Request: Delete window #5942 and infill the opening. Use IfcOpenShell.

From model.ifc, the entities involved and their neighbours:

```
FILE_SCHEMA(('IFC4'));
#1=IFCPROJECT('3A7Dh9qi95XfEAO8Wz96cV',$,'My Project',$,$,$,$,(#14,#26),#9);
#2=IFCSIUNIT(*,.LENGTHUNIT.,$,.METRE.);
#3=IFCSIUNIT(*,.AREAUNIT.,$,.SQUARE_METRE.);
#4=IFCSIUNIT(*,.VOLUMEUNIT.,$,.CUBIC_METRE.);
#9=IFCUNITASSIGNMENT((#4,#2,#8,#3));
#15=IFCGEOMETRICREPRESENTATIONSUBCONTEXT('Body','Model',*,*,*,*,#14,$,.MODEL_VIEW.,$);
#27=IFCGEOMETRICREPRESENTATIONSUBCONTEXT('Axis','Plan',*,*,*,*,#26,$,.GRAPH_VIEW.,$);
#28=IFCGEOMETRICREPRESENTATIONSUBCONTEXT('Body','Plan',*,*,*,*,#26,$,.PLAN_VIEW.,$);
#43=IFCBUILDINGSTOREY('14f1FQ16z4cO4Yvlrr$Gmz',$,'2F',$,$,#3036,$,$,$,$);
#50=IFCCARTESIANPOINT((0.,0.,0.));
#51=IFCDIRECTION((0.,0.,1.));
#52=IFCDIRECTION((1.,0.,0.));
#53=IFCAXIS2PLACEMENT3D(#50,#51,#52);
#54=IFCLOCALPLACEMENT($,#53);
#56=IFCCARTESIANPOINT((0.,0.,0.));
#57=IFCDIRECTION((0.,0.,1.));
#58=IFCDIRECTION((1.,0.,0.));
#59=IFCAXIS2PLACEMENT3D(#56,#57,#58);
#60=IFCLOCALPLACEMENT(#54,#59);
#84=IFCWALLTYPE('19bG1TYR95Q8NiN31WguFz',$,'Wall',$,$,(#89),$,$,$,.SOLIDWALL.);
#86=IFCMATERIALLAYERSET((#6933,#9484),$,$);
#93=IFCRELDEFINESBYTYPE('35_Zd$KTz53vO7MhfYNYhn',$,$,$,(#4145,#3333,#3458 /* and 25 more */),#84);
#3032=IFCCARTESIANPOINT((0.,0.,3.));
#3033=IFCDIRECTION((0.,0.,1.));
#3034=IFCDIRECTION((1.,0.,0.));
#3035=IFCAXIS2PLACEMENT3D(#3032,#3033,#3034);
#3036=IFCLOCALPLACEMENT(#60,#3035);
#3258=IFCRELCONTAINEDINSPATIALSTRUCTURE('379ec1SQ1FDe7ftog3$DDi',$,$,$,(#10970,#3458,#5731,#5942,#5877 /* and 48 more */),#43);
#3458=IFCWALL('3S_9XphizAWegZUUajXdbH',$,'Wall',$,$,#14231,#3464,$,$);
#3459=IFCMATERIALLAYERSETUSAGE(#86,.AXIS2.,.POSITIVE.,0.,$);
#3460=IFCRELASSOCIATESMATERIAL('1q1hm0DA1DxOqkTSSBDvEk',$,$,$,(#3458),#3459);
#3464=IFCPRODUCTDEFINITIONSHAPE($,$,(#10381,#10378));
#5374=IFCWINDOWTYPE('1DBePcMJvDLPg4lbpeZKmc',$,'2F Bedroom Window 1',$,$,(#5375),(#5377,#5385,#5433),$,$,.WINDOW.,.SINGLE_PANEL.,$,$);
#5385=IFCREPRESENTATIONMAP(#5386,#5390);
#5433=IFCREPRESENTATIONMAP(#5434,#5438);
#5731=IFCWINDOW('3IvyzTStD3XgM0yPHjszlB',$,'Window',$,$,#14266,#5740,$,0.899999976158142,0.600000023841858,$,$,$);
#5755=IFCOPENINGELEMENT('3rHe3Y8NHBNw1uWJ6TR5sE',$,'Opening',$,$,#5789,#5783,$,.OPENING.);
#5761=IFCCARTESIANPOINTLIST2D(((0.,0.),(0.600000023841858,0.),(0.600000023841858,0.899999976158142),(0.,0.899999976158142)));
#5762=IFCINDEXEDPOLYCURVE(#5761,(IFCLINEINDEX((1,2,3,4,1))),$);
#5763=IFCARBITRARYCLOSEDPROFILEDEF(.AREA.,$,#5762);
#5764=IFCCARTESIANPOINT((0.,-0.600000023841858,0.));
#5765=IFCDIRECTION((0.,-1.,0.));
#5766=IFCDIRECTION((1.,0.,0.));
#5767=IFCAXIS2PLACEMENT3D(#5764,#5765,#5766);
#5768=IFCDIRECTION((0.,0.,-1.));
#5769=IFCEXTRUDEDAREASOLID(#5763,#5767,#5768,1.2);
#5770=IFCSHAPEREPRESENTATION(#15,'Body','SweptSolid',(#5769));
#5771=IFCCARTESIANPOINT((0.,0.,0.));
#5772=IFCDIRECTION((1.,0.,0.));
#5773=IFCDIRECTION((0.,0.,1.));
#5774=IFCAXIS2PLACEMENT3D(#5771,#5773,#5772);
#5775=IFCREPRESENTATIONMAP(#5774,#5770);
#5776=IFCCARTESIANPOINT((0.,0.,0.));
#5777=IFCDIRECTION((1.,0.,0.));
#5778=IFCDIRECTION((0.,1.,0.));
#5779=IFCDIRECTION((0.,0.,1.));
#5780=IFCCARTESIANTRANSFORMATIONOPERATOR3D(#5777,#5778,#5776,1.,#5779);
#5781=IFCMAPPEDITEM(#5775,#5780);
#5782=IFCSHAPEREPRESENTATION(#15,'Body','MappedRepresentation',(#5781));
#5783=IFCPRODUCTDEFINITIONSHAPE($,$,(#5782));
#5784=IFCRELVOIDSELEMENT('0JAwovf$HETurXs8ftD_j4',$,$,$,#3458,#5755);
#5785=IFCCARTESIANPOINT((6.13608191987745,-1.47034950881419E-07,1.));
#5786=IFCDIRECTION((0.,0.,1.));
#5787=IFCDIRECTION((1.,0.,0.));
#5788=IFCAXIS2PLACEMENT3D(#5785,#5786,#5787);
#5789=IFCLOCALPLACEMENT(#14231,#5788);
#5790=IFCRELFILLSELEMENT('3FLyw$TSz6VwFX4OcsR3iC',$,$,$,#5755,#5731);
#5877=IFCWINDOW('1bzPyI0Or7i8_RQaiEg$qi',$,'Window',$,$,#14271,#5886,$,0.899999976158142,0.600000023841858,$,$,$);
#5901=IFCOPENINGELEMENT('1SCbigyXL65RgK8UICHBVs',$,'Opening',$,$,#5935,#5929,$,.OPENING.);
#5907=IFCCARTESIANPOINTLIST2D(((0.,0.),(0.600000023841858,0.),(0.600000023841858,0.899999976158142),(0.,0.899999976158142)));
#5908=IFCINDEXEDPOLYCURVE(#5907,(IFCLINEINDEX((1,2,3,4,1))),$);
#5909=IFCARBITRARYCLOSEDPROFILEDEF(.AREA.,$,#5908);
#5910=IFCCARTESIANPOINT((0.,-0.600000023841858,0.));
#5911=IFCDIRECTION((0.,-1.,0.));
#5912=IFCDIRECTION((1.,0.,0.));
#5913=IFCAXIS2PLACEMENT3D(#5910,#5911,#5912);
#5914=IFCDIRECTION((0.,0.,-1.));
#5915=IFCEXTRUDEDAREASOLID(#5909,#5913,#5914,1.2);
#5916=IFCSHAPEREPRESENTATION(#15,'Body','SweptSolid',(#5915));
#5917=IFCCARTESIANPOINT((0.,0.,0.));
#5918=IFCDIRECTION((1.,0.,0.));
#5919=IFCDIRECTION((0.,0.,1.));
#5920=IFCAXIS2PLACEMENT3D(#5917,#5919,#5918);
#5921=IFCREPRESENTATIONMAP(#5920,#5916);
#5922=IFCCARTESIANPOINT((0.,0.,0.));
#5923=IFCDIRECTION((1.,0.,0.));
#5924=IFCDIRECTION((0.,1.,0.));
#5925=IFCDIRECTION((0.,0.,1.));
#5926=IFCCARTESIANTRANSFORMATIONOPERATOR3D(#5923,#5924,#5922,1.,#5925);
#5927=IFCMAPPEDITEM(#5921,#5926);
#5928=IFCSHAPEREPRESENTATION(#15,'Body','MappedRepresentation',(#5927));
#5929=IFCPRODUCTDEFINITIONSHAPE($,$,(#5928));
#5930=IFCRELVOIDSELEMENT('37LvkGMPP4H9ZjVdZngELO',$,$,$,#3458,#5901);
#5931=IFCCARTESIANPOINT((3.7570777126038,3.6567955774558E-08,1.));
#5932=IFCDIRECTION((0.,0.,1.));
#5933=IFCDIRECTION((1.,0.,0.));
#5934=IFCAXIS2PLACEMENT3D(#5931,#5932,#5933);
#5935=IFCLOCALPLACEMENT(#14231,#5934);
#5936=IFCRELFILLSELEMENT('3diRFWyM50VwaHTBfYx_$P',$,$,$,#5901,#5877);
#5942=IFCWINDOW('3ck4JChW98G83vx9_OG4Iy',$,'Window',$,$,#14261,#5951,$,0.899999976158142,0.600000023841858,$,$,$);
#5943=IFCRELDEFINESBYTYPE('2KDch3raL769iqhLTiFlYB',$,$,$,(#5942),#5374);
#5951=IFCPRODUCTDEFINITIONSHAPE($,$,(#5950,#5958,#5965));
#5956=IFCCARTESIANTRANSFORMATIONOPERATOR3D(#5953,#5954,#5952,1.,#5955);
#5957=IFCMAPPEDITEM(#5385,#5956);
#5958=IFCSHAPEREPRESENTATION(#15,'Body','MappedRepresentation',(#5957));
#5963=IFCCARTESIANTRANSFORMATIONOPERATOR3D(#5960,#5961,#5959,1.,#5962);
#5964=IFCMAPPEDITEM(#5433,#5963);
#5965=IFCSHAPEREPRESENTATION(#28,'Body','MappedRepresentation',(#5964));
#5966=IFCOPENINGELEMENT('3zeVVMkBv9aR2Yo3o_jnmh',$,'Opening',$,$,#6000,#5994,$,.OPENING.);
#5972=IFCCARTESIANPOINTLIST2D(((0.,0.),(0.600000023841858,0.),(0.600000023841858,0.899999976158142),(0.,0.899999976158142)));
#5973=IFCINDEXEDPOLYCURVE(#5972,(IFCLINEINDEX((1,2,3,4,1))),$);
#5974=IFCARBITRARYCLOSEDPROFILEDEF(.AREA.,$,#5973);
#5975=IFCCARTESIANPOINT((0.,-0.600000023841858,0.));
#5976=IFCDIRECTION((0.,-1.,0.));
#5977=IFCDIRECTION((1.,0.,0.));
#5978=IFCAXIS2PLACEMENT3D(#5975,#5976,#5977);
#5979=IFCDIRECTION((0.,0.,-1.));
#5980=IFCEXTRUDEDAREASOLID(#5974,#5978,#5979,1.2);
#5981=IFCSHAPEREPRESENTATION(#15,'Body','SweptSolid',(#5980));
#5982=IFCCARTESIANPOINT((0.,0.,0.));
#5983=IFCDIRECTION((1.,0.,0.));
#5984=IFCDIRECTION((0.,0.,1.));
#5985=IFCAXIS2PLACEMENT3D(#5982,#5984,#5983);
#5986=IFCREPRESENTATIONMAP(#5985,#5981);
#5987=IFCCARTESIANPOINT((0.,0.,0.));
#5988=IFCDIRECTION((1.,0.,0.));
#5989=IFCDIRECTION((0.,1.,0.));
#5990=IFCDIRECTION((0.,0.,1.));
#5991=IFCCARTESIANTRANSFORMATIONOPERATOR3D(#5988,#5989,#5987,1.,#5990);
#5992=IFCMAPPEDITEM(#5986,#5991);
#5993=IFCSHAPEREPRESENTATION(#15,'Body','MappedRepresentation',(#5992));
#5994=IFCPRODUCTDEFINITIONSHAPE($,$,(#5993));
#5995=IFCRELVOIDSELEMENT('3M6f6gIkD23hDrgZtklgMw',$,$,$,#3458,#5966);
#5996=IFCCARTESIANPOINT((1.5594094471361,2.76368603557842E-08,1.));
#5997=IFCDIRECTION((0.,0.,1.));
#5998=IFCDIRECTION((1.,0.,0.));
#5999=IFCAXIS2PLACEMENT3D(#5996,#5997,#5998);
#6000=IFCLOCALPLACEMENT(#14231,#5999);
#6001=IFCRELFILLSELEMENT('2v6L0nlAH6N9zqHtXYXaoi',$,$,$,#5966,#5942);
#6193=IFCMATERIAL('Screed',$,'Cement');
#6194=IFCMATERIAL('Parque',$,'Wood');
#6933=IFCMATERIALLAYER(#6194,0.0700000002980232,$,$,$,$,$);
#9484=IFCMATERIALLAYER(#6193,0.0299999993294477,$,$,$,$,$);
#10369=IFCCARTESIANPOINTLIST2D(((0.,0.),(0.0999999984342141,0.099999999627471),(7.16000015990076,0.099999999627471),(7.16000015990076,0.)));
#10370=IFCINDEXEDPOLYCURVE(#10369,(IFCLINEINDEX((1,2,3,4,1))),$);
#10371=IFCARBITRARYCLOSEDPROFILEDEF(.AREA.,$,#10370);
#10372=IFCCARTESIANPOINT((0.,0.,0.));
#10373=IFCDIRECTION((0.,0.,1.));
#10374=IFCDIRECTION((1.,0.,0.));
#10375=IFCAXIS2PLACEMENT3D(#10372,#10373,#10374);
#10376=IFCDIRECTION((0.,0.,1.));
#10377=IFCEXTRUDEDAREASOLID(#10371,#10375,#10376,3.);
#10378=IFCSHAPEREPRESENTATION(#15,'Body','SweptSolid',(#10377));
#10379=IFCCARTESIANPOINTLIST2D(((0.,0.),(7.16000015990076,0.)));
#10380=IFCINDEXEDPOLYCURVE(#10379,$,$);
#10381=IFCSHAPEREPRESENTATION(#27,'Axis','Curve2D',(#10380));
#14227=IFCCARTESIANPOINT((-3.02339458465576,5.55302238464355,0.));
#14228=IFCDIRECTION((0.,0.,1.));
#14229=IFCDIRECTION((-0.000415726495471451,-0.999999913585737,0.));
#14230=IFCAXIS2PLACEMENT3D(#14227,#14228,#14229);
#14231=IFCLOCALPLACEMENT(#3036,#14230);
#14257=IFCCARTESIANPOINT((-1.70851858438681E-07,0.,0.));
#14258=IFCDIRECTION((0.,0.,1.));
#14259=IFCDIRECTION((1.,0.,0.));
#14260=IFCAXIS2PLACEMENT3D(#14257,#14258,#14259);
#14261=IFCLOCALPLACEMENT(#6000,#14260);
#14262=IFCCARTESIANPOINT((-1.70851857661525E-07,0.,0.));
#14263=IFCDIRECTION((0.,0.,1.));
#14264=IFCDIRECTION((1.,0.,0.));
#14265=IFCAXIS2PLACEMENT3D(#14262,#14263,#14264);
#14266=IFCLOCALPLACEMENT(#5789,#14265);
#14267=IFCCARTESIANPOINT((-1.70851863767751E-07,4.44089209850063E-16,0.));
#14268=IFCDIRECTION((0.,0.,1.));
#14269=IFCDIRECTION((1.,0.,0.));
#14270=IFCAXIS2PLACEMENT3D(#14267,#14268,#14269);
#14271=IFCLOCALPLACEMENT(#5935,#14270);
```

```python
import ifcopenshell
import ifcopenshell.api.feature
import ifcopenshell.api.root
import ifcopenshell.geom
import ifcopenshell.util.shape

model = ifcopenshell.open("model.ifc")
settings = ifcopenshell.geom.settings()


def volume(element):
    """Net volume in cubic metres, openings subtracted."""
    shape = ifcopenshell.geom.create_shape(settings, element)
    return ifcopenshell.util.shape.get_volume(shape.geometry)


window = model.by_guid("3ck4JChW98G83vx9_OG4Iy")
opening = window.FillsVoids[0].RelatingOpeningElement
wall = opening.VoidsElements[0].RelatingBuildingElement
before = volume(wall)

ifcopenshell.api.root.remove_product(model, product=window)
ifcopenshell.api.feature.remove_feature(model, feature=opening)

after = volume(wall)

print(f"wall volume {before:.3f} -> {after:.3f} m3")

model.write("model_rev.ifc")
```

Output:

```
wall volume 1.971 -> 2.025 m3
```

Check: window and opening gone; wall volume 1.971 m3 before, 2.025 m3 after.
